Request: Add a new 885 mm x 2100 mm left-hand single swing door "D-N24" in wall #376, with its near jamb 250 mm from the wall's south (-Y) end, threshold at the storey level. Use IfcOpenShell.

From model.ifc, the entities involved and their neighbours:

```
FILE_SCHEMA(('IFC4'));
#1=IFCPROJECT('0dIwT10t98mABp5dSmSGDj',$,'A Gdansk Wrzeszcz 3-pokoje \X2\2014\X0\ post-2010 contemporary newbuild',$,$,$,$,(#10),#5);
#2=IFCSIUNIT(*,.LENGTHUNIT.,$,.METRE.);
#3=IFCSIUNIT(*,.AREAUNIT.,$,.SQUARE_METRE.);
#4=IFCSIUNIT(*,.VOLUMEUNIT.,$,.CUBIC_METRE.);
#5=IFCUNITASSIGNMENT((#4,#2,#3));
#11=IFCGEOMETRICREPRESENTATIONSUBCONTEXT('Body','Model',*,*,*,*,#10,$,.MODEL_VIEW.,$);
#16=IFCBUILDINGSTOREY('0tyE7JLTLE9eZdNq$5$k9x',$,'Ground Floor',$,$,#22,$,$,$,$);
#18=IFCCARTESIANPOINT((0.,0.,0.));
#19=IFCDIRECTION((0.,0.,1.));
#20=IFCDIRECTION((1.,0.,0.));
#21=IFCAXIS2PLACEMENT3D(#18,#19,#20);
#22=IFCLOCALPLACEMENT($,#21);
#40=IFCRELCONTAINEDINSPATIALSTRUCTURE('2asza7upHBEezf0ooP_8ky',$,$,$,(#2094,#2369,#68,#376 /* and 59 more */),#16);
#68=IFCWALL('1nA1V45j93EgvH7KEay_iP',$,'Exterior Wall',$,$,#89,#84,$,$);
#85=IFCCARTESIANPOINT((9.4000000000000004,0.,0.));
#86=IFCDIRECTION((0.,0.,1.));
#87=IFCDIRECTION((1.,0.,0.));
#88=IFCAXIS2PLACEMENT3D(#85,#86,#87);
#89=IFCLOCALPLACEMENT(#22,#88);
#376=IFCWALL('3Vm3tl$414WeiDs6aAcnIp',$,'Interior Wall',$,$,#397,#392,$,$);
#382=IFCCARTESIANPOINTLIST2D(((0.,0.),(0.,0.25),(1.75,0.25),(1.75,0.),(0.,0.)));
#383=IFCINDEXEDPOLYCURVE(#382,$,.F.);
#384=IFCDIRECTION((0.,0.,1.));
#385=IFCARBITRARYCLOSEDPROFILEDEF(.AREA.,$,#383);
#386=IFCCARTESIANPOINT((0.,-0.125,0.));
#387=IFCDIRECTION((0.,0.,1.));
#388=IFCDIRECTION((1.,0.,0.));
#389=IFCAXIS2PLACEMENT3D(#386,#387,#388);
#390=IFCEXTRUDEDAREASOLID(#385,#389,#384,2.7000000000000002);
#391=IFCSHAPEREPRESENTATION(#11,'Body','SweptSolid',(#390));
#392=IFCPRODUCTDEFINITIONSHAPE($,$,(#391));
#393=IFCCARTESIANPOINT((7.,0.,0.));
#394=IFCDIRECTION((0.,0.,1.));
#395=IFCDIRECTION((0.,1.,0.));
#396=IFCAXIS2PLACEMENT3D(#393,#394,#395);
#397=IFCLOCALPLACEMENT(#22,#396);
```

```python
import numpy as np
import ifcopenshell
import ifcopenshell.api.feature
import ifcopenshell.api.geometry
import ifcopenshell.api.root
import ifcopenshell.api.spatial
import ifcopenshell.geom
import ifcopenshell.util.element
import ifcopenshell.util.placement
import ifcopenshell.util.representation
import ifcopenshell.util.shape
import ifcopenshell.util.unit

model = ifcopenshell.open("model.ifc")
unit_scale = ifcopenshell.util.unit.calculate_unit_scale(model)
settings = ifcopenshell.geom.settings()


def volume(element):
    """Net volume in cubic metres, openings subtracted."""
    shape = ifcopenshell.geom.create_shape(settings, element)
    return ifcopenshell.util.shape.get_volume(shape.geometry)


wall = model.by_id(376)
storey = ifcopenshell.util.element.get_container(wall, ifc_class="IfcBuildingStorey")
context = ifcopenshell.util.representation.get_context(model, "Model", "Body", "MODEL_VIEW")
before = volume(wall)

width, height, from_end, sill = 0.885, 2.1, 0.25, 0.0  # metres

# The wall runs along its own X axis, and the end named is its -X end.
wall_shape = ifcopenshell.geom.create_shape(settings, wall)
x, y, z = ifcopenshell.util.shape.get_vertices(wall_shape.geometry).T
start = x.min() + from_end
face, thickness = float(y.min()), float(y.max() - y.min())
wall_matrix = ifcopenshell.util.placement.get_local_placement(wall.ObjectPlacement)
level = ifcopenshell.util.placement.get_local_placement(storey.ObjectPlacement)[2, 3]


def in_wall(x, y):
    """Placement at x, y metres in the wall's axes, at sill height."""
    matrix = wall_matrix.copy()
    matrix[:, 3] = wall_matrix @ np.array([x / unit_scale, y / unit_scale, 0.0, 1.0])
    matrix[2, 3] = level + sill / unit_scale
    return matrix


# Opening: a box that overshoots both wall faces by 50 mm.
opening = ifcopenshell.api.root.create_entity(model, ifc_class="IfcOpeningElement", predefined_type="OPENING")
box = ifcopenshell.api.geometry.add_wall_representation(
    model, context=context, length=width, height=height, thickness=thickness + 0.1
)
ifcopenshell.api.geometry.assign_representation(model, product=opening, representation=box)
ifcopenshell.api.geometry.edit_object_placement(model, product=opening, matrix=in_wall(start, face - 0.05), is_si=False)
ifcopenshell.api.feature.add_feature(model, feature=opening, element=wall)

door = ifcopenshell.api.root.create_entity(model, ifc_class="IfcDoor", name="D-N24", predefined_type="DOOR")
door.OverallWidth, door.OverallHeight = width / unit_scale, height / unit_scale
door.OperationType = "SINGLE_SWING_LEFT"
body = ifcopenshell.api.geometry.add_door_representation(
    model,
    context=context,
    overall_width=door.OverallWidth,
    overall_height=door.OverallHeight,
    operation_type="SINGLE_SWING_LEFT",
    lining_properties={"LiningDepth": thickness / unit_scale, "ThresholdDepth": thickness / unit_scale},
)
ifcopenshell.api.geometry.assign_representation(model, product=door, representation=body)
ifcopenshell.api.spatial.assign_container(model, products=[door], relating_structure=storey)
ifcopenshell.api.feature.add_filling(model, opening=opening, element=door)

# The lining spans the wall, so the door starts at the wall face.
ifcopenshell.api.geometry.edit_object_placement(model, product=door, matrix=in_wall(start, face), is_si=False)

after = volume(wall)

print(f"wall volume {before:.3f} -> {after:.3f} m3")

model.write("model-out.ifc")
```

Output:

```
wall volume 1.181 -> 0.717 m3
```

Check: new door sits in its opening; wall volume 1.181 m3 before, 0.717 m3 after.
